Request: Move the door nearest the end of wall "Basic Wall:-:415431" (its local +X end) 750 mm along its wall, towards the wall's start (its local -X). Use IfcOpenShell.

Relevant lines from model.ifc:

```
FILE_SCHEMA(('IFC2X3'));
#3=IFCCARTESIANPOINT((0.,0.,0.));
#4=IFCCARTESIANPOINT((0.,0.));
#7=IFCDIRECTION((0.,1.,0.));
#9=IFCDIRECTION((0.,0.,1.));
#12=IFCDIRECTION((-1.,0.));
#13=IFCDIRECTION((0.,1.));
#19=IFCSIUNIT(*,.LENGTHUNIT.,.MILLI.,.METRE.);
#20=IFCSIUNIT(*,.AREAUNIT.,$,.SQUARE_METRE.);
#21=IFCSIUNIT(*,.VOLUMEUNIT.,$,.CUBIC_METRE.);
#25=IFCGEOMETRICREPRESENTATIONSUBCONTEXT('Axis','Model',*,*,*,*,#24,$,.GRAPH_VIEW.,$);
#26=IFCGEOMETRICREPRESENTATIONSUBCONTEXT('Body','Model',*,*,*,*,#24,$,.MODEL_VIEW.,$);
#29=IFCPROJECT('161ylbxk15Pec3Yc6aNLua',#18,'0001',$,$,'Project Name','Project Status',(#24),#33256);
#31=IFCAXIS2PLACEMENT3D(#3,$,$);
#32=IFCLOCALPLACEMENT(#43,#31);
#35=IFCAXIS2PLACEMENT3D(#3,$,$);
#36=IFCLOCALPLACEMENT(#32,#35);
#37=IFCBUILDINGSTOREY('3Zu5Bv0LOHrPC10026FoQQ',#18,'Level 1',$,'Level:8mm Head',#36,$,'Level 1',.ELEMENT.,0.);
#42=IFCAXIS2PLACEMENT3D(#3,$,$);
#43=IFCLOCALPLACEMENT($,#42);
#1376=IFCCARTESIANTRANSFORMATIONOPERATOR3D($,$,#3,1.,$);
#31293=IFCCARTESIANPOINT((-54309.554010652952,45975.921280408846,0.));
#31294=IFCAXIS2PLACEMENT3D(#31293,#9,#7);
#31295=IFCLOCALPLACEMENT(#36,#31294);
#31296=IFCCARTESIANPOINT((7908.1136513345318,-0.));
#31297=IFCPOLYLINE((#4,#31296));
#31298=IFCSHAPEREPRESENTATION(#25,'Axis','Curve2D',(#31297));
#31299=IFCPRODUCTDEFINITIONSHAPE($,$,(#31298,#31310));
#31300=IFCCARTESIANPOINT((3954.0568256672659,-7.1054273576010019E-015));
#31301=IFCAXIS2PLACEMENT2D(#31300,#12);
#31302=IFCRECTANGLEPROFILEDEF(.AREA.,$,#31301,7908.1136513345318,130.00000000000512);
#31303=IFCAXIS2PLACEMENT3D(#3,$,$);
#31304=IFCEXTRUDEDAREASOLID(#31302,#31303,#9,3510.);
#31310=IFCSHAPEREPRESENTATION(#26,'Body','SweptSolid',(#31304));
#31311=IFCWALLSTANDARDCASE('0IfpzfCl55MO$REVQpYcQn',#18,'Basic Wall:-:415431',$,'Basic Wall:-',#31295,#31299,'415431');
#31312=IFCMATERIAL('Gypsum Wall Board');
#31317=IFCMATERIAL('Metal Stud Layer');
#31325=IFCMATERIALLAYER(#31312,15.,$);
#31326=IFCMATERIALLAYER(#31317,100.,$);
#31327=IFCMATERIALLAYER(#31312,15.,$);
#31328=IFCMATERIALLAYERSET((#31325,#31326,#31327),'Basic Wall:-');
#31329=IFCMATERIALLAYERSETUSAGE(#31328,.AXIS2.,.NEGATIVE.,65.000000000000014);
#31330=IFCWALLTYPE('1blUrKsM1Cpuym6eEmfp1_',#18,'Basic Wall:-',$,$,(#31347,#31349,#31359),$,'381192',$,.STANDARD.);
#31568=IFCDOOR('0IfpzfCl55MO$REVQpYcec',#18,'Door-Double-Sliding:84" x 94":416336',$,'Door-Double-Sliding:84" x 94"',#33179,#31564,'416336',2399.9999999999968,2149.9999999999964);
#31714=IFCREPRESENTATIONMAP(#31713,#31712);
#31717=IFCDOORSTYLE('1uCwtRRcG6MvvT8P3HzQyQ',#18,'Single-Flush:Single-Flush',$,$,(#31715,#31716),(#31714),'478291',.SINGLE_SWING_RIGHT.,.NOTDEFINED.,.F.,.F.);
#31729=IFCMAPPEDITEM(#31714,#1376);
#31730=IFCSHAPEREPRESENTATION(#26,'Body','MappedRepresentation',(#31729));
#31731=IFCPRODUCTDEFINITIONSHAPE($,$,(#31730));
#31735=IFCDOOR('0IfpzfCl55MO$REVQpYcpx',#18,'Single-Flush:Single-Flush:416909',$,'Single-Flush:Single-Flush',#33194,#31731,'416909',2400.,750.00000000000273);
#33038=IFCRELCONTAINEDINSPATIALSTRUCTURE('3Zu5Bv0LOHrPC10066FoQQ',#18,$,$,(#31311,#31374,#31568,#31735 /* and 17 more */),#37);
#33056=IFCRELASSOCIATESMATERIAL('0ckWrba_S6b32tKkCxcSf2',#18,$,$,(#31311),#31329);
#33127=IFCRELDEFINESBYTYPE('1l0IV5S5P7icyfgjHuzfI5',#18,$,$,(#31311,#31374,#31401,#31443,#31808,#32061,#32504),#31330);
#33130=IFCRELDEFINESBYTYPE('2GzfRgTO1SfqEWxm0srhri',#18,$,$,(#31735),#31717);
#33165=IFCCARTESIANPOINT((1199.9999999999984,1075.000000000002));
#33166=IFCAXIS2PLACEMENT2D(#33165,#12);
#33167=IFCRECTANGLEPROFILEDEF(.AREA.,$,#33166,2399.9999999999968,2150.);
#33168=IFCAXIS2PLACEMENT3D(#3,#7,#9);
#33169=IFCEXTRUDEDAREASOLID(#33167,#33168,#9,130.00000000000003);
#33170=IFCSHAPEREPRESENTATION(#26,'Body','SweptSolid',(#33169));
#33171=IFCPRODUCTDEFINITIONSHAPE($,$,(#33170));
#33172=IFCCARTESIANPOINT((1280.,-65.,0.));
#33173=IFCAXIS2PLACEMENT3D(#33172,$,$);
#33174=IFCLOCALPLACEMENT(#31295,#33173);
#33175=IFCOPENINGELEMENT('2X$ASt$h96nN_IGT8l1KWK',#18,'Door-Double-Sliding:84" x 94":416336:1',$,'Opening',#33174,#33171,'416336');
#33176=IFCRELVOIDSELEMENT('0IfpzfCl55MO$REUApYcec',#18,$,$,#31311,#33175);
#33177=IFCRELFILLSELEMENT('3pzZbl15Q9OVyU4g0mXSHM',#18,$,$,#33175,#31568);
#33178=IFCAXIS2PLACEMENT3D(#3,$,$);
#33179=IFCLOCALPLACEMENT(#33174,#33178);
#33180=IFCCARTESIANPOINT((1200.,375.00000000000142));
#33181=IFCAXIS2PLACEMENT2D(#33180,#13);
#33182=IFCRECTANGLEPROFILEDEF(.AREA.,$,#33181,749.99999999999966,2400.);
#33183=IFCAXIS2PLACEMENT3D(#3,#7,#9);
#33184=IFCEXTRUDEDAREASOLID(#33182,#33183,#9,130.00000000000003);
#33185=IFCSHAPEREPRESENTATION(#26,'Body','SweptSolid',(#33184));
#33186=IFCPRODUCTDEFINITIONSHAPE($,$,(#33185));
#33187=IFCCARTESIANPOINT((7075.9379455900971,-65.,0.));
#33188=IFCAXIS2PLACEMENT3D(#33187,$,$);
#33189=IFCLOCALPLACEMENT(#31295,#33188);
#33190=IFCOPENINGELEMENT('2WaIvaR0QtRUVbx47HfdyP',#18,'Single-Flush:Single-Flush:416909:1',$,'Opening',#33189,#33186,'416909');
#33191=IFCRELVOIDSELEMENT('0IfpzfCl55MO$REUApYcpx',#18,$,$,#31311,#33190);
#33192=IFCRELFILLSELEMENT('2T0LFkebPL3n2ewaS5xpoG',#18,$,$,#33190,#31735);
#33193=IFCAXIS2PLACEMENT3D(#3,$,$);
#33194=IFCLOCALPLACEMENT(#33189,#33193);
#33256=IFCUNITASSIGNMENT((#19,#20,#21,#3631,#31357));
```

```python
import ifcopenshell
import ifcopenshell.api.geometry
import ifcopenshell.util.placement

model = ifcopenshell.open("model.ifc")

door = model.by_guid("0IfpzfCl55MO$REVQpYcpx")
opening = door.FillsVoids[0].RelatingOpeningElement
wall = opening.VoidsElements[0].RelatingBuildingElement

wall_matrix = ifcopenshell.util.placement.get_local_placement(wall.ObjectPlacement)
shift = wall_matrix[:3, 0] * -750.0
before = ifcopenshell.util.placement.get_local_placement(door.ObjectPlacement)[:3, 3].copy()

# The door is placed relative to its opening, so it follows when the opening moves.
matrix = ifcopenshell.util.placement.get_local_placement(opening.ObjectPlacement)
matrix[:3, 3] += shift
ifcopenshell.api.geometry.edit_object_placement(
    model, product=opening, matrix=matrix, is_si=False, should_transform_children=True
)

after = ifcopenshell.util.placement.get_local_placement(door.ObjectPlacement)[:3, 3]
print("door moved by", (after - before).round(3) + 0.0)

model.write("model_updated.ifc")
```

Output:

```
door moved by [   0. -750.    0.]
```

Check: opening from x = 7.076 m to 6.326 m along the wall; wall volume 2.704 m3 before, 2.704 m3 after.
